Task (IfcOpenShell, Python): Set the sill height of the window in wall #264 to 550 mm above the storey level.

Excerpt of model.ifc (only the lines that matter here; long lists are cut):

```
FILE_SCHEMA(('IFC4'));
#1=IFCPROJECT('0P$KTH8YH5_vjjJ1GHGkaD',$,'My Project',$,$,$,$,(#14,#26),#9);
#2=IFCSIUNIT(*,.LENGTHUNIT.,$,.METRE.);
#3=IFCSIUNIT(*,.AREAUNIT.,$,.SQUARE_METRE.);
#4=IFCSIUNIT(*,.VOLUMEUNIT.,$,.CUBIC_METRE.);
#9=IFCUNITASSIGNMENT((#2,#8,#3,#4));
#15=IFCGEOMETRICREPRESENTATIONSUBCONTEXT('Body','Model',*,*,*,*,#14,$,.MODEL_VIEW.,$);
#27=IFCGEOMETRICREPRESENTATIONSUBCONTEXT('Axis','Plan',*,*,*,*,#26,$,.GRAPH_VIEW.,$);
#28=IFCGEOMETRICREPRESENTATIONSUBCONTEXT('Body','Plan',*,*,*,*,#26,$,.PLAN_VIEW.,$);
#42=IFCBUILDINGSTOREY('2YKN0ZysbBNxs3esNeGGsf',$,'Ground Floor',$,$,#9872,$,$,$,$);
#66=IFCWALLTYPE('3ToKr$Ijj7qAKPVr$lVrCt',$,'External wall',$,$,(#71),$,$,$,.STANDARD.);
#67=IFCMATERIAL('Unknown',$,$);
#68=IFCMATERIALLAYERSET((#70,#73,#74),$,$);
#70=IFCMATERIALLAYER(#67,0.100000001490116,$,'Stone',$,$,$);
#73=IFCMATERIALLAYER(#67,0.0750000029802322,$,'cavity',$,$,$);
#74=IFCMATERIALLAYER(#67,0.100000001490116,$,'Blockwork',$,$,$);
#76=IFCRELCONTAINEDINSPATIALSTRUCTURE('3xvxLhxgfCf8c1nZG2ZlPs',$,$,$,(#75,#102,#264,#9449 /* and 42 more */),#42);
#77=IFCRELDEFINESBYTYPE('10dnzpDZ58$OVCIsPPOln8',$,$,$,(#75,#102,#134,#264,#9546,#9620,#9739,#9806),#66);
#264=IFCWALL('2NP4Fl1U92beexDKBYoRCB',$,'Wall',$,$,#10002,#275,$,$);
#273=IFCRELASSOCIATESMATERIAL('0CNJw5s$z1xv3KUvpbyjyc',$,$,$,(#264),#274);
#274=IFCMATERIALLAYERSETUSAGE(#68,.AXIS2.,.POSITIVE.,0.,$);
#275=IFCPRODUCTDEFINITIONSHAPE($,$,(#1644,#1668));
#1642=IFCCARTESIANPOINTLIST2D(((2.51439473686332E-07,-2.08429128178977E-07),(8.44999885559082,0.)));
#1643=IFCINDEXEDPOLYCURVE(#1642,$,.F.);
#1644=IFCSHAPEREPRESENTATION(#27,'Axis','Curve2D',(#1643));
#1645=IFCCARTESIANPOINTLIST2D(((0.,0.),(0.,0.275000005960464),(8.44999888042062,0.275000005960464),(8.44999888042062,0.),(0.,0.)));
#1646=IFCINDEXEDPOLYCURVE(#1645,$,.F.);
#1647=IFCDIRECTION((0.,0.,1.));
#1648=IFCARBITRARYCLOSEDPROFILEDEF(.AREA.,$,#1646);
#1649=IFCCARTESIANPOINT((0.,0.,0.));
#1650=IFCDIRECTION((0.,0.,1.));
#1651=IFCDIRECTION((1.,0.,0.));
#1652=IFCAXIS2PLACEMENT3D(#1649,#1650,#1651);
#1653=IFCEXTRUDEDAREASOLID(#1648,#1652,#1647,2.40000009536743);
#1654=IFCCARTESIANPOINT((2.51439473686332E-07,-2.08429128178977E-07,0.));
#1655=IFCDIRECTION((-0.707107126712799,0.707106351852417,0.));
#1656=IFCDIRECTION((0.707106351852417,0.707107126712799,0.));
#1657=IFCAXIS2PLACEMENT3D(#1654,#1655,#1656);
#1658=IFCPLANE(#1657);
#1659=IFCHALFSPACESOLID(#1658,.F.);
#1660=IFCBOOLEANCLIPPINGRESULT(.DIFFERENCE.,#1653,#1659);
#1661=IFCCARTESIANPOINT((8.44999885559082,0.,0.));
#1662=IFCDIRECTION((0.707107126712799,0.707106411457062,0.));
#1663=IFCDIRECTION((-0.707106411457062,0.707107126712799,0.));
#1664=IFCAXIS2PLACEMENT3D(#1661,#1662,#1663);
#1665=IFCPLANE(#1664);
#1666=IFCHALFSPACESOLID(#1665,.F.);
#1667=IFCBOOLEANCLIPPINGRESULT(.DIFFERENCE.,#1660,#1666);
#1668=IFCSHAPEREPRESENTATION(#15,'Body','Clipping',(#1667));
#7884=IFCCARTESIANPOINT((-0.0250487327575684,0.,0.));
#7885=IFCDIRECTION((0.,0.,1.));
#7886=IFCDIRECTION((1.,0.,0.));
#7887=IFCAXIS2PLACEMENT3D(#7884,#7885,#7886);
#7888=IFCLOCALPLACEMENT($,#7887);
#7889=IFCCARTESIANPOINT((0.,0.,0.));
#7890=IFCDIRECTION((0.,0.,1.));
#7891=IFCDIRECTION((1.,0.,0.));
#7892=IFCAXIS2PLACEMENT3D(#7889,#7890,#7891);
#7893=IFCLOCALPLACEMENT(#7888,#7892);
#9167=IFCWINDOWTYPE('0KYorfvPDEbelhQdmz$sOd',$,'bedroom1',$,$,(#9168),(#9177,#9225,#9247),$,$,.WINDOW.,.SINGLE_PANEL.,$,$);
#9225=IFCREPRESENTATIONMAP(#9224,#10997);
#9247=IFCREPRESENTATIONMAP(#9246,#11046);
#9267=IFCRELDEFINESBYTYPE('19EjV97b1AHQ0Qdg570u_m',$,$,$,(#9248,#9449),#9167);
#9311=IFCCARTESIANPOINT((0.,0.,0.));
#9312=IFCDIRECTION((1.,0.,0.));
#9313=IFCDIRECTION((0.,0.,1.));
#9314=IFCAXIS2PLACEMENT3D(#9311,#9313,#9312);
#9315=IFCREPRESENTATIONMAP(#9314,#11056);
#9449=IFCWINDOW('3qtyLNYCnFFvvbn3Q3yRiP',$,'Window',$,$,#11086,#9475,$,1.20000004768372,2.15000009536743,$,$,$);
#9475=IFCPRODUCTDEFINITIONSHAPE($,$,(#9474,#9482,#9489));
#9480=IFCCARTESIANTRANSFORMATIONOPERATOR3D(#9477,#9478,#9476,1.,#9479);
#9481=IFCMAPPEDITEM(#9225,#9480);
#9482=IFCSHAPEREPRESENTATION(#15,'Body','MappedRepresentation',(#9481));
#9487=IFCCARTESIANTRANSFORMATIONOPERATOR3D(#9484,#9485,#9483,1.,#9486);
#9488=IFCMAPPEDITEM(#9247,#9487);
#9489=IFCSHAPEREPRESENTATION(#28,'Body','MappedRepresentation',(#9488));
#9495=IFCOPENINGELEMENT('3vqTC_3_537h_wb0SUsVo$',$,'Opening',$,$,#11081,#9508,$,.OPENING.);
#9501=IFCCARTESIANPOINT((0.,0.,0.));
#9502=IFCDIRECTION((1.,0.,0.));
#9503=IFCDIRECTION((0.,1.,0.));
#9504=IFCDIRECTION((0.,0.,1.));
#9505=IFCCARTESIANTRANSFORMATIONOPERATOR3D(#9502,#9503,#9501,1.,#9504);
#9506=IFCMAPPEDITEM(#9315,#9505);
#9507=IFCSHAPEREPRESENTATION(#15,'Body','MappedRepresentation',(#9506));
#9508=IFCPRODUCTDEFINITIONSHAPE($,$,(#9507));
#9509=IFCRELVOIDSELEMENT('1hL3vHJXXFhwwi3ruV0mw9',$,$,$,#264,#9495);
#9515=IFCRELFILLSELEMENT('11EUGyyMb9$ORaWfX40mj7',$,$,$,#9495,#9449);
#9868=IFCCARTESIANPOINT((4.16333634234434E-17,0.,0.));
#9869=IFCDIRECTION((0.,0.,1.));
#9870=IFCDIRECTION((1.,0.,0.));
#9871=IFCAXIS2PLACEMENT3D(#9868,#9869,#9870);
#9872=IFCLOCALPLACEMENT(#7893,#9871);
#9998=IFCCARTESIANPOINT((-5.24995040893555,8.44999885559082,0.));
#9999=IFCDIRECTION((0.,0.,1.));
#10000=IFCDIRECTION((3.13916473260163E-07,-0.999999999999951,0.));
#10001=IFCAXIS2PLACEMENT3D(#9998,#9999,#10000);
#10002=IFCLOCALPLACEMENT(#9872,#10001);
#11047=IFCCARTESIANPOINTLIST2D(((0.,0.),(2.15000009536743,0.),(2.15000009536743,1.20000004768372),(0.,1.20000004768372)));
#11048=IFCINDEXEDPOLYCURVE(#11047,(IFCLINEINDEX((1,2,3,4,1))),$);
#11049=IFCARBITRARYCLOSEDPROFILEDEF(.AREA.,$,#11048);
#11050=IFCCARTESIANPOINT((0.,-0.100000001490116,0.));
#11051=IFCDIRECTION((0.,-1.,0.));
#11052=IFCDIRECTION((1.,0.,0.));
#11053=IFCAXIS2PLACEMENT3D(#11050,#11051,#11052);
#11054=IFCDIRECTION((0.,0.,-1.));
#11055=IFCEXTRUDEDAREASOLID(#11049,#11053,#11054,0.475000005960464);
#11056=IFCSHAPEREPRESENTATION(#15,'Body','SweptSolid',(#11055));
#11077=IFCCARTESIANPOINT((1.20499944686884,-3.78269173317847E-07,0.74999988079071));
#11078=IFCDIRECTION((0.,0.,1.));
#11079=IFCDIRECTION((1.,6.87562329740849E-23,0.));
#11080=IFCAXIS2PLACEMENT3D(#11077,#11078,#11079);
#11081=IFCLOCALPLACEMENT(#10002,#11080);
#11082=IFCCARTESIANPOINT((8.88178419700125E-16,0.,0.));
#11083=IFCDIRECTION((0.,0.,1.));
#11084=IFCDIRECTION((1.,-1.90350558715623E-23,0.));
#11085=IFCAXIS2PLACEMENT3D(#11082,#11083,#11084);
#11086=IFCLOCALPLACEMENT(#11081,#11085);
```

```python
import numpy as np
import ifcopenshell
import ifcopenshell.api.geometry
import ifcopenshell.geom
import ifcopenshell.util.element
import ifcopenshell.util.placement
import ifcopenshell.util.shape
import ifcopenshell.util.unit

model = ifcopenshell.open("model.ifc")
unit_scale = ifcopenshell.util.unit.calculate_unit_scale(model)

window = model.by_id(9449)
opening = window.FillsVoids[0].RelatingOpeningElement
storey = ifcopenshell.util.element.get_container(window, ifc_class="IfcBuildingStorey")
level = ifcopenshell.util.placement.get_local_placement(storey.ObjectPlacement)[2, 3]

# The opening's origin need not be at the sill, so measure its lowest point.
shape = ifcopenshell.geom.create_shape(ifcopenshell.geom.settings(), opening)
bottom = ifcopenshell.util.shape.get_shape_bottom_elevation(shape, shape.geometry) / unit_scale
dz = level + 0.55 - bottom

shift = np.array([0.0, 0.0, dz])
# The window is placed relative to its opening, so it follows when the opening moves.
matrix = ifcopenshell.util.placement.get_local_placement(opening.ObjectPlacement)
matrix[:3, 3] += shift
ifcopenshell.api.geometry.edit_object_placement(
    model, product=opening, matrix=matrix, is_si=False, should_transform_children=True
)

print(f"moved by {dz * unit_scale:+.3f} m")

model.write("model_edited.ifc")
```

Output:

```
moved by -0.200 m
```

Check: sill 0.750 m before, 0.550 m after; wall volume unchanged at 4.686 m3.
